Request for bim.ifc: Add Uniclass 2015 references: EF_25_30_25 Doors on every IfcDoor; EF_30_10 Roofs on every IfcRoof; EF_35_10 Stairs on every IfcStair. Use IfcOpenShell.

First a look at what the model holds.

```python
import ifcopenshell

model = ifcopenshell.open("bim.ifc")
print(model.schema)
print("classifications:", [c.Name for c in model.by_type("IfcClassification")])
for ifc_class in ("IfcDoor", "IfcRoof", "IfcStair", "IfcWall", "IfcWindow"):
    print(ifc_class, len(model.by_type(ifc_class)))
```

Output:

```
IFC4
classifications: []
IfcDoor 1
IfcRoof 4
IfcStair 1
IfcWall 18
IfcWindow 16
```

```python
import ifcopenshell
import ifcopenshell.api.classification

model = ifcopenshell.open("bim.ifc")

system = ifcopenshell.api.classification.add_classification(model, classification="Uniclass 2015")

codes = {
    "IfcDoor": ("EF_25_30_25", "Doors"),
    "IfcRoof": ("EF_30_10", "Roofs"),
    "IfcStair": ("EF_35_10", "Stairs"),
}
for ifc_class, (code, name) in codes.items():
    products = model.by_type(ifc_class)
    ifcopenshell.api.classification.add_reference(
        model, products=products, classification=system, identification=code, name=name
    )
    print(code, len(products))

model.write("bim-out.ifc")
```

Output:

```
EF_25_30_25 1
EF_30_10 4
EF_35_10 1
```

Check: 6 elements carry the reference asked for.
